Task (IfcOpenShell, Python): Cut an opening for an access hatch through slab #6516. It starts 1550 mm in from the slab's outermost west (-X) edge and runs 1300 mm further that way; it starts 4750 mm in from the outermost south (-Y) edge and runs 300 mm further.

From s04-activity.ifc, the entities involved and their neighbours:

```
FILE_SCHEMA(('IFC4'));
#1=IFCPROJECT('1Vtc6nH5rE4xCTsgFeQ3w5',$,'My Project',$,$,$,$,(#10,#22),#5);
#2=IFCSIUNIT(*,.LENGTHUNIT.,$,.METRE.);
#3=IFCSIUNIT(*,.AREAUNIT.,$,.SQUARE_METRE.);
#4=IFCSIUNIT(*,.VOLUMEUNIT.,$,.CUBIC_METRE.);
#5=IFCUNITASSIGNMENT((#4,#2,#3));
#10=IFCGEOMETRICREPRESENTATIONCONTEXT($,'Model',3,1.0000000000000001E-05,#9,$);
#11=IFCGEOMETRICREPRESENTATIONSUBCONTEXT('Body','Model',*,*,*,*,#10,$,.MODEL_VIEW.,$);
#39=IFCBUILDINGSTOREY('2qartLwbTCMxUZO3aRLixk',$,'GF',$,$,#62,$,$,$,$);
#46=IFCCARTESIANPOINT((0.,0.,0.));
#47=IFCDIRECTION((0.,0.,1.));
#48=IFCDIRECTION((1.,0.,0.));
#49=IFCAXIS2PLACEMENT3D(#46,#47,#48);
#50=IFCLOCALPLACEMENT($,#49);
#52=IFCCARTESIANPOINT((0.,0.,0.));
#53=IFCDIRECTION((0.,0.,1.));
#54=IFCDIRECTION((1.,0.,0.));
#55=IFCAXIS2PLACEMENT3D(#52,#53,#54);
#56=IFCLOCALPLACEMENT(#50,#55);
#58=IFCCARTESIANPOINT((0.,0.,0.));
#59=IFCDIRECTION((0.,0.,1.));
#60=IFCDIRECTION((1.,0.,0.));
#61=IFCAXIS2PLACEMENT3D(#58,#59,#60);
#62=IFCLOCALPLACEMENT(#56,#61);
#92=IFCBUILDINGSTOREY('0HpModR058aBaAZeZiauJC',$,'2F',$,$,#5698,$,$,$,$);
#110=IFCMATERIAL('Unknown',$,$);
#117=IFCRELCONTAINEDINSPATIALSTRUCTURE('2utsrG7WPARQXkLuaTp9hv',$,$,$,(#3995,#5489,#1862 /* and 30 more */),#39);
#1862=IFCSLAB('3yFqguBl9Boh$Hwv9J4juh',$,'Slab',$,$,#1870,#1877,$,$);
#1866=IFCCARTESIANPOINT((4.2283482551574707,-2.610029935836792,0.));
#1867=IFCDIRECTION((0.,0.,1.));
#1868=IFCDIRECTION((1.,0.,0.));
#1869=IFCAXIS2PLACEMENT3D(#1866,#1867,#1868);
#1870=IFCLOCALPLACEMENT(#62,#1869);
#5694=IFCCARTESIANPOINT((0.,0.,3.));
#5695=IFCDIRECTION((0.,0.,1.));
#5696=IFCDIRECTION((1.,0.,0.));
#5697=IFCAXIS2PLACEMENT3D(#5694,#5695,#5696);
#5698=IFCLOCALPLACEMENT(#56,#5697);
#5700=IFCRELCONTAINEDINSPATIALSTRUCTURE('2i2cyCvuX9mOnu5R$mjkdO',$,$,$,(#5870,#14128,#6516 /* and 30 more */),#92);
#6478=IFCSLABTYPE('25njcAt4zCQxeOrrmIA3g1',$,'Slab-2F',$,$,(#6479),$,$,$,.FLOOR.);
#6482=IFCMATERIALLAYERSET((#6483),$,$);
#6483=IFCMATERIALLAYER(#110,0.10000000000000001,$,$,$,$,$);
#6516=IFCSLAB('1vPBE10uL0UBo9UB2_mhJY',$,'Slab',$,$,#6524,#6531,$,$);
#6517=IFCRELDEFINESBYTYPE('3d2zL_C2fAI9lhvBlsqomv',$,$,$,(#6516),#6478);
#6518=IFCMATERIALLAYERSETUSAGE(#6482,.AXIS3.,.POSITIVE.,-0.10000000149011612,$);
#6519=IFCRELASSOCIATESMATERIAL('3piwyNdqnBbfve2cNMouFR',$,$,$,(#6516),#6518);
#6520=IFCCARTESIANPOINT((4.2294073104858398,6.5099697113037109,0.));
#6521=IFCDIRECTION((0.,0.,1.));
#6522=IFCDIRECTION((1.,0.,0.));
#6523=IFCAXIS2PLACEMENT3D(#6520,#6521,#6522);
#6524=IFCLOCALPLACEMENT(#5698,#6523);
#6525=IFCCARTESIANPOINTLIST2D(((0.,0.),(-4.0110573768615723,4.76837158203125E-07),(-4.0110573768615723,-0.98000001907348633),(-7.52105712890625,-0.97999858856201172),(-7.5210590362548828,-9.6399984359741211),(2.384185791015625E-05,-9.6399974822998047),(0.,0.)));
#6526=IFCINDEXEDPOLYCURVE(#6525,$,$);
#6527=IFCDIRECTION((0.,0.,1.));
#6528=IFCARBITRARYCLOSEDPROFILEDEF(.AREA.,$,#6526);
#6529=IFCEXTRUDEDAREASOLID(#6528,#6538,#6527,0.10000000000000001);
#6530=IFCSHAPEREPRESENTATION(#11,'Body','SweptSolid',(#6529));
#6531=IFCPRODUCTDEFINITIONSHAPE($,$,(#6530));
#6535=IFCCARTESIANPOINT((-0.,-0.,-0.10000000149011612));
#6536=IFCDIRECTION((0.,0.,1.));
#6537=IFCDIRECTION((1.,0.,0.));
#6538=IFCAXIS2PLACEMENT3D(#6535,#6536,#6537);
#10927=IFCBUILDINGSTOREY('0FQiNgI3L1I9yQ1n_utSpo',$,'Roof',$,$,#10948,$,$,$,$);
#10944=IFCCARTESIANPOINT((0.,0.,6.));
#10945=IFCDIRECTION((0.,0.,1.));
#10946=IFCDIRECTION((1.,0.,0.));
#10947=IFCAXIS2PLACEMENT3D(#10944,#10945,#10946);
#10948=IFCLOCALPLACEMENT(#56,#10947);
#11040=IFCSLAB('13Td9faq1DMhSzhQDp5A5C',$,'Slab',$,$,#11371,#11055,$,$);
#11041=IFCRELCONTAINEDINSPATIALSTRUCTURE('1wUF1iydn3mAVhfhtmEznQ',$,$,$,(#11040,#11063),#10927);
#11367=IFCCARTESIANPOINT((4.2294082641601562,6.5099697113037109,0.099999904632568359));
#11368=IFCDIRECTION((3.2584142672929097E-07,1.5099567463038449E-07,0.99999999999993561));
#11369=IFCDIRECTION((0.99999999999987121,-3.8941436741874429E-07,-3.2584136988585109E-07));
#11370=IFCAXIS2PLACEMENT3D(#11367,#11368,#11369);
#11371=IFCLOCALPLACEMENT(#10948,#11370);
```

```python
import numpy as np
import ifcopenshell
import ifcopenshell.api.feature
import ifcopenshell.api.geometry
import ifcopenshell.api.root
import ifcopenshell.geom
import ifcopenshell.util.placement
import ifcopenshell.util.representation
import ifcopenshell.util.shape
import ifcopenshell.util.unit

model = ifcopenshell.open("s04-activity.ifc")
unit_scale = ifcopenshell.util.unit.calculate_unit_scale(model)
settings = ifcopenshell.geom.settings()


def volume(element):
    """Net volume in cubic metres, openings subtracted."""
    shape = ifcopenshell.geom.create_shape(settings, element)
    return ifcopenshell.util.shape.get_volume(shape.geometry)


slab = model.by_guid("1vPBE10uL0UBo9UB2_mhJY")
before = volume(slab)

# Extent in the slab's own axes, in metres. The edges named are its -X and -Y sides.
slab_shape = ifcopenshell.geom.create_shape(settings, slab)
vertices = ifcopenshell.util.shape.get_vertices(slab_shape.geometry)
x_min, y_min, bottom = vertices.min(axis=0)
top = vertices[:, 2].max()

opening = ifcopenshell.api.root.create_entity(model, ifc_class="IfcOpeningElement", name="Access hatch opening", predefined_type="OPENING")
context = ifcopenshell.util.representation.get_context(model, "Model", "Body", "MODEL_VIEW")
width, depth = 1.3, 0.3
outline = [(0.0, 0.0), (width, 0.0), (width, depth), (0.0, depth), (0.0, 0.0)]
# Overshoot both faces by 50 mm so the cut is clean.
shape = ifcopenshell.api.geometry.add_slab_representation(
    model, context=context, depth=top - bottom + 0.1, polyline=outline
)
ifcopenshell.api.geometry.assign_representation(model, product=opening, representation=shape)

matrix = ifcopenshell.util.placement.get_local_placement(slab.ObjectPlacement)
matrix[:, 3] = matrix @ np.append(np.array([x_min + 1.55, y_min + 4.75, bottom - 0.05]) / unit_scale, 1.0)
ifcopenshell.api.geometry.edit_object_placement(model, product=opening, matrix=matrix, is_si=False)
ifcopenshell.api.feature.add_feature(model, feature=opening, element=slab)

after = volume(slab)

print(f"slab volume {before:.3f} -> {after:.3f} m3")

model.write("s04-activity_v2.ifc")
```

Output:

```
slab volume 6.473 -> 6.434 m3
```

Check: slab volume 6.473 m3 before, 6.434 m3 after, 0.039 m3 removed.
